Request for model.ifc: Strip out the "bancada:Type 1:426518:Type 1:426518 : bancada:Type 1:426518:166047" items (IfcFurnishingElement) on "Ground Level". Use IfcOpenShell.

First a look at what the model holds.

```python
import ifcopenshell
import ifcopenshell.util.element

model = ifcopenshell.open("model.ifc")
print(model.schema)
storey = next(s for s in model.by_type("IfcBuildingStorey") if s.Name == "Ground Level")
furniture = [e for e in ifcopenshell.util.element.get_decomposition(storey) if e.is_a("IfcFurnishingElement")]
seen = {}
for e in furniture:
    element_type = ifcopenshell.util.element.get_type(e)
    name = element_type.Name if element_type not in (None, e) else None
    seen[name] = seen.get(name, 0) + 1
for name, count in sorted(seen.items(), key=str):
    print(count, "x", name)
```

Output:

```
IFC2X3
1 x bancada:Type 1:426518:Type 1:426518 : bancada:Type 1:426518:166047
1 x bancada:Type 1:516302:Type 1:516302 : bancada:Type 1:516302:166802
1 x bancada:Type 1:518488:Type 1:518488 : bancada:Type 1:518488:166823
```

```python
import ifcopenshell
import ifcopenshell.api.root
import ifcopenshell.util.element

model = ifcopenshell.open("model.ifc")

storey = next(s for s in model.by_type("IfcBuildingStorey") if s.Name == "Ground Level")
furniture = [e for e in ifcopenshell.util.element.get_decomposition(storey) if e.is_a("IfcFurnishingElement")]
targets = [e for e in furniture if (t := ifcopenshell.util.element.get_type(e)) not in (None, e) and t.Name == "bancada:Type 1:426518:Type 1:426518 : bancada:Type 1:426518:166047"]

for e in targets:
    ifcopenshell.api.root.remove_product(model, product=e)
print(len(targets), "removed")

model.write("model-out.ifc")
```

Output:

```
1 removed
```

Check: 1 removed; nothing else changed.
